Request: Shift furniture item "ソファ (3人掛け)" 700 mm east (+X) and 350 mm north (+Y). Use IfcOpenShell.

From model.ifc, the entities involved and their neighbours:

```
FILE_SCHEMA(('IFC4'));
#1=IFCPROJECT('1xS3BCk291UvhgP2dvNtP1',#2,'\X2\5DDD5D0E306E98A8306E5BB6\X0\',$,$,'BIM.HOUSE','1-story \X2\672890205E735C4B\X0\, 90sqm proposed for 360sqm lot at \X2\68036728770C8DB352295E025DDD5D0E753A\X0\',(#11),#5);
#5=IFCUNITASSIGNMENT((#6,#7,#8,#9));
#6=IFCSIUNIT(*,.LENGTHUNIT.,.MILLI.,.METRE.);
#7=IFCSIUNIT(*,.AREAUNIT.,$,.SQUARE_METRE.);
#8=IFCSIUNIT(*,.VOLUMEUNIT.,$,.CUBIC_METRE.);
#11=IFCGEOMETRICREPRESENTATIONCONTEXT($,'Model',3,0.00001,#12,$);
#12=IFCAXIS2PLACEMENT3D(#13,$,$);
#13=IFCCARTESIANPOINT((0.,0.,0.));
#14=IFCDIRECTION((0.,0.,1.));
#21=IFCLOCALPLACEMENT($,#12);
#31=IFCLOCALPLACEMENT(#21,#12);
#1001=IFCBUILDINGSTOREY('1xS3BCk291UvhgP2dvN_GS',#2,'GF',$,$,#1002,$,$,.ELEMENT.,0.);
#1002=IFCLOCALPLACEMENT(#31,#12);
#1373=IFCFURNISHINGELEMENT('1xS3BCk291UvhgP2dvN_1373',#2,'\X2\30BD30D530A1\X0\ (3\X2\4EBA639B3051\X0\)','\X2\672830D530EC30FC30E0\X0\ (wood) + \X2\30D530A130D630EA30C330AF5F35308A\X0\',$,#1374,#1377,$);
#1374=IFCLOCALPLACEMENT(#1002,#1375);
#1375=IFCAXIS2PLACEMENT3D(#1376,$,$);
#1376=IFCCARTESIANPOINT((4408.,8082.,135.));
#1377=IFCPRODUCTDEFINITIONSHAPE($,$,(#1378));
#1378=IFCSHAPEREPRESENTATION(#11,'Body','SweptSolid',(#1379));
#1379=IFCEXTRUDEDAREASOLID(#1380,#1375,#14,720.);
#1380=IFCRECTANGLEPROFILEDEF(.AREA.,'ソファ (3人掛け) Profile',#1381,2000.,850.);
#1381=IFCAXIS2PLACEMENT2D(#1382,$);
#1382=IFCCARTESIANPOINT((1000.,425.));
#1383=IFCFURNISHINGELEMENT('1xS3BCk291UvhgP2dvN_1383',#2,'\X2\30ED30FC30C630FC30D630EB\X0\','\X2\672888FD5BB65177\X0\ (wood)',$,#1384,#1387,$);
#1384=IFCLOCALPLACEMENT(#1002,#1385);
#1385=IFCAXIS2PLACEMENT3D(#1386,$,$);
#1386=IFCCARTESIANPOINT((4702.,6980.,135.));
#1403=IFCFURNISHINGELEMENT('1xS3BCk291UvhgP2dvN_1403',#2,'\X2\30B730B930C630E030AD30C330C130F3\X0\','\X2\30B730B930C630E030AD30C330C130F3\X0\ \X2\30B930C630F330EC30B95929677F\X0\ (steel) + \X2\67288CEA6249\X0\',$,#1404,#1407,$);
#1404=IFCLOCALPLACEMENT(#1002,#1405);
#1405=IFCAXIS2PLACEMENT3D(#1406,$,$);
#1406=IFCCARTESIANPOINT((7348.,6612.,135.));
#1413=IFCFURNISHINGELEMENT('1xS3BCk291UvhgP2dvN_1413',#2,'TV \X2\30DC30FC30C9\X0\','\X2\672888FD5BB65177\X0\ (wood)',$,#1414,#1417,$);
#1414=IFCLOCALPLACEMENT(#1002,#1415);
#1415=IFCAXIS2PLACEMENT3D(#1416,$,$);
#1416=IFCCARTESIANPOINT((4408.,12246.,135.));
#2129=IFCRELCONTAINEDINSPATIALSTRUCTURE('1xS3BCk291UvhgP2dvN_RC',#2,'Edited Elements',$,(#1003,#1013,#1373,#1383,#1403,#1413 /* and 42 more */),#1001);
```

```python
import ifcopenshell
import ifcopenshell.api.geometry
import ifcopenshell.util.placement

model = ifcopenshell.open("model.ifc")

item = model.by_guid("1xS3BCk291UvhgP2dvN_1373")
matrix = ifcopenshell.util.placement.get_local_placement(item.ObjectPlacement)
matrix[0, 3] += 700.0
matrix[1, 3] += 350.0
ifcopenshell.api.geometry.edit_object_placement(model, product=item, matrix=matrix, is_si=False)

print(ifcopenshell.util.placement.get_local_placement(item.ObjectPlacement).round(3) + 0.0)

model.write("model-out.ifc")
```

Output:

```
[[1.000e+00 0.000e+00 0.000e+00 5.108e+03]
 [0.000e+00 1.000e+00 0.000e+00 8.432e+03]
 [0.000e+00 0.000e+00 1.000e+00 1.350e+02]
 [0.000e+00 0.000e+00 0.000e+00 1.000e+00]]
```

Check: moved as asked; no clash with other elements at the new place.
